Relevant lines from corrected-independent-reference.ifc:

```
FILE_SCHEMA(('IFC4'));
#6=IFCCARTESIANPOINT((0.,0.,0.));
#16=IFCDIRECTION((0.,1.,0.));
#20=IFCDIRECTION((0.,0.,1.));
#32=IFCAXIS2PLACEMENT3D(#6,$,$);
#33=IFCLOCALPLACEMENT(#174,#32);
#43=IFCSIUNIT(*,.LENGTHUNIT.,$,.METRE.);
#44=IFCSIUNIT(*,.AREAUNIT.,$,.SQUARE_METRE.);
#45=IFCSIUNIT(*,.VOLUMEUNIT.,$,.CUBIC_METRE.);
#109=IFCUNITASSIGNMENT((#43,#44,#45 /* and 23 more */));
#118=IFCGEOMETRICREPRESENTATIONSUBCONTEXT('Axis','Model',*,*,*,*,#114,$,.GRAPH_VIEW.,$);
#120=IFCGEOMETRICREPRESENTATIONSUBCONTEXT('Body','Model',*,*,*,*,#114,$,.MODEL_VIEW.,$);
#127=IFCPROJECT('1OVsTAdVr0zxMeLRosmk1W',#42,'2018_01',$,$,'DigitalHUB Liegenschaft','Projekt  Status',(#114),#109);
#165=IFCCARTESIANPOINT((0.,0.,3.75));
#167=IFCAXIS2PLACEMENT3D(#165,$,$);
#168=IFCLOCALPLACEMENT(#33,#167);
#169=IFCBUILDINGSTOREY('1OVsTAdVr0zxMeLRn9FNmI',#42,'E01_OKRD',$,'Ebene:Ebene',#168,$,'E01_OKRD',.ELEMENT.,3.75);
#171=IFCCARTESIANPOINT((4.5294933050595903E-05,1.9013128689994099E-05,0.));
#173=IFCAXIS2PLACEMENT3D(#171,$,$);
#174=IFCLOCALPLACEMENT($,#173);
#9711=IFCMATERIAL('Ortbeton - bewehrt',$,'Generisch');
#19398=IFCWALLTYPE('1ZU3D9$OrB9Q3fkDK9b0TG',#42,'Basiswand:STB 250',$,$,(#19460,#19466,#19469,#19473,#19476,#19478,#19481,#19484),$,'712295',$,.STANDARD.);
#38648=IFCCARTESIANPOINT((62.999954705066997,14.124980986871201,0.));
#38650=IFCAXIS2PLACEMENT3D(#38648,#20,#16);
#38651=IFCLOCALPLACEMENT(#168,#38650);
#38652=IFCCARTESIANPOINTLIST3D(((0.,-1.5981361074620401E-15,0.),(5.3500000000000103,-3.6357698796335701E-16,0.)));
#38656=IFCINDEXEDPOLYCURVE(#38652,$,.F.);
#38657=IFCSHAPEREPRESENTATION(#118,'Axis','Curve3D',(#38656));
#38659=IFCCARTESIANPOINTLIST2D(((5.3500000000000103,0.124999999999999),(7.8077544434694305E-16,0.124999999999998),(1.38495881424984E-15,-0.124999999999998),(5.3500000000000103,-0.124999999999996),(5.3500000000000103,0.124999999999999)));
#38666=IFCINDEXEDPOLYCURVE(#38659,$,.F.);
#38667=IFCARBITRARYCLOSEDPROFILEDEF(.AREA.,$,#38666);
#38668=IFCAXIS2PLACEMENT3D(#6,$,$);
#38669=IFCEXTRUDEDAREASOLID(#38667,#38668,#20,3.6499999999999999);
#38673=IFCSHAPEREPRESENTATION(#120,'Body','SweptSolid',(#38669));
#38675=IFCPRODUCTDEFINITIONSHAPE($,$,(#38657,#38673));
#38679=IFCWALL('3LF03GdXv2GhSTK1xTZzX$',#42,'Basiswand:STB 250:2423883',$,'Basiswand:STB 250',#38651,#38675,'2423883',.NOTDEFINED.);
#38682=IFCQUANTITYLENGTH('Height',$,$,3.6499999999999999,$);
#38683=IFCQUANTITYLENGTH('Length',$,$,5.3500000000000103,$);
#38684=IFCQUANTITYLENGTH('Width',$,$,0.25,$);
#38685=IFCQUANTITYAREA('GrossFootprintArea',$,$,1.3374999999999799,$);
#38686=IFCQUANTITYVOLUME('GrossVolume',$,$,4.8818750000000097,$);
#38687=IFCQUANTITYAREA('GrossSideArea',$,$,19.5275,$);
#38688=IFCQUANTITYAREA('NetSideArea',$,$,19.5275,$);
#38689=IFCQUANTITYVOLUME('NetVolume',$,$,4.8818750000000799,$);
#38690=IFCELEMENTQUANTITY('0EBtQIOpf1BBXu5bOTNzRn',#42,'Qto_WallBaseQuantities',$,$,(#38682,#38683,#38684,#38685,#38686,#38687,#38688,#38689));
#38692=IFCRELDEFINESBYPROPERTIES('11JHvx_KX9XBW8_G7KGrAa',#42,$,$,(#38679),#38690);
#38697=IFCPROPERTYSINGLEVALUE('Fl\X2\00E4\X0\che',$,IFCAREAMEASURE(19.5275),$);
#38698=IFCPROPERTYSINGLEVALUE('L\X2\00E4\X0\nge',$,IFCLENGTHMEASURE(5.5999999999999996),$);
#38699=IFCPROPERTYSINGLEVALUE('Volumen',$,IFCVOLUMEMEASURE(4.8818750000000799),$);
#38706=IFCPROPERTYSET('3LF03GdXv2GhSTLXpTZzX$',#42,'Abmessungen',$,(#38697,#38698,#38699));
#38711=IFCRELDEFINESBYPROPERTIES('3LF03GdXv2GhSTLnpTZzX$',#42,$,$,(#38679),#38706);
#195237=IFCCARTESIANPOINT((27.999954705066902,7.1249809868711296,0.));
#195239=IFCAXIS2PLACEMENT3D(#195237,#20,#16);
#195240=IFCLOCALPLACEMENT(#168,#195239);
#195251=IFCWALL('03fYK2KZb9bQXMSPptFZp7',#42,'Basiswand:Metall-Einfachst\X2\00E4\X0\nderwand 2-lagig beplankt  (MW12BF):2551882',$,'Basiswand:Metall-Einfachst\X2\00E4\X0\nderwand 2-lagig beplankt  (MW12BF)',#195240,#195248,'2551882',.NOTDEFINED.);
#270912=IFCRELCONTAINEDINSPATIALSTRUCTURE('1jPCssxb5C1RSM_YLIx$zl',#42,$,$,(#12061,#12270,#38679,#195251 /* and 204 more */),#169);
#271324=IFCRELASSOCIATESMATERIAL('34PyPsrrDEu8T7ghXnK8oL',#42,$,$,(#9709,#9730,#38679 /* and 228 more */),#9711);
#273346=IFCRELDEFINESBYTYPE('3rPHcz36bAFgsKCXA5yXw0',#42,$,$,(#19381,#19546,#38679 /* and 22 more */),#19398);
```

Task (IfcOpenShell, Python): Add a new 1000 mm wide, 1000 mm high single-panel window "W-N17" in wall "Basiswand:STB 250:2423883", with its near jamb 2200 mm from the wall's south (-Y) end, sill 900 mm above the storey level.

```python
import numpy as np
import ifcopenshell
import ifcopenshell.api.feature
import ifcopenshell.api.geometry
import ifcopenshell.api.pset
import ifcopenshell.api.root
import ifcopenshell.api.spatial
import ifcopenshell.geom
import ifcopenshell.util.element
import ifcopenshell.util.placement
import ifcopenshell.util.representation
import ifcopenshell.util.shape
import ifcopenshell.util.unit

model = ifcopenshell.open("corrected-independent-reference.ifc")
unit_scale = ifcopenshell.util.unit.calculate_unit_scale(model)
area_scale = ifcopenshell.util.unit.calculate_unit_scale(model, "AREAUNIT")
volume_scale = ifcopenshell.util.unit.calculate_unit_scale(model, "VOLUMEUNIT")
settings = ifcopenshell.geom.settings()


def volume(element):
    """Net volume in cubic metres, openings subtracted."""
    shape = ifcopenshell.geom.create_shape(settings, element)
    return ifcopenshell.util.shape.get_volume(shape.geometry)


wall = model.by_id(38679)
storey = ifcopenshell.util.element.get_container(wall, ifc_class="IfcBuildingStorey")
context = ifcopenshell.util.representation.get_context(model, "Model", "Body", "MODEL_VIEW")
before = volume(wall)

width, height, from_end, sill = 1, 1, 2.2, 0.9  # metres

# The wall runs along its own X axis, and the end named is its -X end.
wall_shape = ifcopenshell.geom.create_shape(settings, wall)
x, y, z = ifcopenshell.util.shape.get_vertices(wall_shape.geometry).T
start = x.min() + from_end
face, thickness = float(y.min()), float(y.max() - y.min())
wall_matrix = ifcopenshell.util.placement.get_local_placement(wall.ObjectPlacement)
level = ifcopenshell.util.placement.get_local_placement(storey.ObjectPlacement)[2, 3]


def in_wall(x, y):
    """Placement at x, y metres in the wall's axes, at sill height."""
    matrix = wall_matrix.copy()
    matrix[:, 3] = wall_matrix @ np.array([x / unit_scale, y / unit_scale, 0.0, 1.0])
    matrix[2, 3] = level + sill / unit_scale
    return matrix


# Opening: a box that overshoots both wall faces by 50 mm.
opening = ifcopenshell.api.root.create_entity(model, ifc_class="IfcOpeningElement", predefined_type="OPENING")
box = ifcopenshell.api.geometry.add_wall_representation(
    model, context=context, length=width, height=height, thickness=thickness + 0.1
)
ifcopenshell.api.geometry.assign_representation(model, product=opening, representation=box)
ifcopenshell.api.geometry.edit_object_placement(model, product=opening, matrix=in_wall(start, face - 0.05), is_si=False)
ifcopenshell.api.feature.add_feature(model, feature=opening, element=wall)

window = ifcopenshell.api.root.create_entity(model, ifc_class="IfcWindow", name="W-N17", predefined_type="WINDOW")
window.OverallWidth, window.OverallHeight = width / unit_scale, height / unit_scale
window.PartitioningType = "SINGLE_PANEL"
body = ifcopenshell.api.geometry.add_window_representation(
    model,
    context=context,
    overall_width=window.OverallWidth,
    overall_height=window.OverallHeight,
    partition_type="SINGLE_PANEL",
)
ifcopenshell.api.geometry.assign_representation(model, product=window, representation=body)
ifcopenshell.api.spatial.assign_container(model, products=[window], relating_structure=storey)
ifcopenshell.api.feature.add_filling(model, opening=opening, element=window)

# Centre the window in the wall's thickness.
ifcopenshell.api.geometry.edit_object_placement(model, product=window, matrix=in_wall(start, face), is_si=False)
window_shape = ifcopenshell.geom.create_shape(settings, window)
depth = ifcopenshell.util.shape.get_vertices(window_shape.geometry)[:, 1]
offset = face + thickness / 2 - (depth.min() + depth.max()) / 2
ifcopenshell.api.geometry.edit_object_placement(model, product=window, matrix=in_wall(start, offset), is_si=False)

after = volume(wall)

# Update the wall's stored quantities.
qto = model.by_id(ifcopenshell.util.element.get_pset(wall, "Qto_WallBaseQuantities", should_inherit=False)["id"])
ifcopenshell.api.pset.edit_qto(model, qto=qto, properties={
    "NetSideArea": after / thickness / area_scale,
    "NetVolume": after / volume_scale,
})
pset = model.by_id(ifcopenshell.util.element.get_pset(wall, "Abmessungen", should_inherit=False)["id"])
ifcopenshell.api.pset.edit_pset(model, pset=pset, properties={
    "Fläche": model.create_entity("IfcAreaMeasure", after / thickness / area_scale),
    "Volumen": model.create_entity("IfcVolumeMeasure", after / volume_scale),
})

print(f"wall volume {before:.3f} -> {after:.3f} m3")

model.write("corrected-independent-reference_edited.ifc")
```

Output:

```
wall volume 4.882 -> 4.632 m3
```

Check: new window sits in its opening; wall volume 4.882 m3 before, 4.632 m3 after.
